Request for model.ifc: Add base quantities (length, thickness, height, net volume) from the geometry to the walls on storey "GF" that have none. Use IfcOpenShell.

First a look at what the model holds.

```python
import ifcopenshell
import ifcopenshell.util.element
import ifcopenshell.util.unit

model = ifcopenshell.open("model.ifc")
print(model.schema)
for unit_type in ("LENGTHUNIT", "AREAUNIT", "VOLUMEUNIT"):
    print(unit_type, ifcopenshell.util.unit.calculate_unit_scale(model, unit_type))
storey = next(s for s in model.by_type("IfcBuildingStorey") if s.Name == "GF")
walls = [e for e in ifcopenshell.util.element.get_decomposition(storey) if e.is_a("IfcWall")]
for e in sorted(walls, key=lambda e: e.id()):
    print(e.id(), e.is_a(), e.Name, list(ifcopenshell.util.element.get_psets(e, qtos_only=True)), sep=" | ")
```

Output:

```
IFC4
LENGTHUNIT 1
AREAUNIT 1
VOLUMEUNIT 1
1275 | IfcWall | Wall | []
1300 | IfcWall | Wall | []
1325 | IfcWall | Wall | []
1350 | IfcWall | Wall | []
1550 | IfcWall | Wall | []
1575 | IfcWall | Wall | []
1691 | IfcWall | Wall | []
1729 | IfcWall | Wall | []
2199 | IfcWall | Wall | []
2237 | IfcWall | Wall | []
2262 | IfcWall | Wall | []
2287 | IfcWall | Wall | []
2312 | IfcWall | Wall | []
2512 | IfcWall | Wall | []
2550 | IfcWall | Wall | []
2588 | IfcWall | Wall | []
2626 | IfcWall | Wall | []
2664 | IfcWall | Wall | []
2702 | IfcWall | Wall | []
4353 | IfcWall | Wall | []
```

```python
import ifcopenshell
import ifcopenshell.api.pset
import ifcopenshell.geom
import ifcopenshell.util.element
import ifcopenshell.util.shape
import ifcopenshell.util.unit

model = ifcopenshell.open("model.ifc")
unit_scale = ifcopenshell.util.unit.calculate_unit_scale(model)
volume_scale = ifcopenshell.util.unit.calculate_unit_scale(model, "VOLUMEUNIT")
settings = ifcopenshell.geom.settings()

storey = next(s for s in model.by_type("IfcBuildingStorey") if s.Name == "GF")
walls = [e for e in ifcopenshell.util.element.get_decomposition(storey) if e.is_a("IfcWall")]

for e in sorted(walls, key=lambda e: e.id()):
    if ifcopenshell.util.element.get_psets(e, qtos_only=True, should_inherit=False):
        continue
    # Geometry comes back in metres, in the element's own axes.
    shape = ifcopenshell.geom.create_shape(settings, e)
    values = {
        "Length": ifcopenshell.util.shape.get_x(shape.geometry) / unit_scale,
        "Width": ifcopenshell.util.shape.get_y(shape.geometry) / unit_scale,
        "Height": ifcopenshell.util.shape.get_z(shape.geometry) / unit_scale,
        "NetVolume": ifcopenshell.util.shape.get_volume(shape.geometry) / volume_scale,
    }
    qto = ifcopenshell.api.pset.add_qto(model, product=e, name="Qto_WallBaseQuantities")
    ifcopenshell.api.pset.edit_qto(model, qto=qto, properties=values)
    print(e.id(), {k: round(v, 3) for k, v in values.items()})

model.write("model-out.ifc")
```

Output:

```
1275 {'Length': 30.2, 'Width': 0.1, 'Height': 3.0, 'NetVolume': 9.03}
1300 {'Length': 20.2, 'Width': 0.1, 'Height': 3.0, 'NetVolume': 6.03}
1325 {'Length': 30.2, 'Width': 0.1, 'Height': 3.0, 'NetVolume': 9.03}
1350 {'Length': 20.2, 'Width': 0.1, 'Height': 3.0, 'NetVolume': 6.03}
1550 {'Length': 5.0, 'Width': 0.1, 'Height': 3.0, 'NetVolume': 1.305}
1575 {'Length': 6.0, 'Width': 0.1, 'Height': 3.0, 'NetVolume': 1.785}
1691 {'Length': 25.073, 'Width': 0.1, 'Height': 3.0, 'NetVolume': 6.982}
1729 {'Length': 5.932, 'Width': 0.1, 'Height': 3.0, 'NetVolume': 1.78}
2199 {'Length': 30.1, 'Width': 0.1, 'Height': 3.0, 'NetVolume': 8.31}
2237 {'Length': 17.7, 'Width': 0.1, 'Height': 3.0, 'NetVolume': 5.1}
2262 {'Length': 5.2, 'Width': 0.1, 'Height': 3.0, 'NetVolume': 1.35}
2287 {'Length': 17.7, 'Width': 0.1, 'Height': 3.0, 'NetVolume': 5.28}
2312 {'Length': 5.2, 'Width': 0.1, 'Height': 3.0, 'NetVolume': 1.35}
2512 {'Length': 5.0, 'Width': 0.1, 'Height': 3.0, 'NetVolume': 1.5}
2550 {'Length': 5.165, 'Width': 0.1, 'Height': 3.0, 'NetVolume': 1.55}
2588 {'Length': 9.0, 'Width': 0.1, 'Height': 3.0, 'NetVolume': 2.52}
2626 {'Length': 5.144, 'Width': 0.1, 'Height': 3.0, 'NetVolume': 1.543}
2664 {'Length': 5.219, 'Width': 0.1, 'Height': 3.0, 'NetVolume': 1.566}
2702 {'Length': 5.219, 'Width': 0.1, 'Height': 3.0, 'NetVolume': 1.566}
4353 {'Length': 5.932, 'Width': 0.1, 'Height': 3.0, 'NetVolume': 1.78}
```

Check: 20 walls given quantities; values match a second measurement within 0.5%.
